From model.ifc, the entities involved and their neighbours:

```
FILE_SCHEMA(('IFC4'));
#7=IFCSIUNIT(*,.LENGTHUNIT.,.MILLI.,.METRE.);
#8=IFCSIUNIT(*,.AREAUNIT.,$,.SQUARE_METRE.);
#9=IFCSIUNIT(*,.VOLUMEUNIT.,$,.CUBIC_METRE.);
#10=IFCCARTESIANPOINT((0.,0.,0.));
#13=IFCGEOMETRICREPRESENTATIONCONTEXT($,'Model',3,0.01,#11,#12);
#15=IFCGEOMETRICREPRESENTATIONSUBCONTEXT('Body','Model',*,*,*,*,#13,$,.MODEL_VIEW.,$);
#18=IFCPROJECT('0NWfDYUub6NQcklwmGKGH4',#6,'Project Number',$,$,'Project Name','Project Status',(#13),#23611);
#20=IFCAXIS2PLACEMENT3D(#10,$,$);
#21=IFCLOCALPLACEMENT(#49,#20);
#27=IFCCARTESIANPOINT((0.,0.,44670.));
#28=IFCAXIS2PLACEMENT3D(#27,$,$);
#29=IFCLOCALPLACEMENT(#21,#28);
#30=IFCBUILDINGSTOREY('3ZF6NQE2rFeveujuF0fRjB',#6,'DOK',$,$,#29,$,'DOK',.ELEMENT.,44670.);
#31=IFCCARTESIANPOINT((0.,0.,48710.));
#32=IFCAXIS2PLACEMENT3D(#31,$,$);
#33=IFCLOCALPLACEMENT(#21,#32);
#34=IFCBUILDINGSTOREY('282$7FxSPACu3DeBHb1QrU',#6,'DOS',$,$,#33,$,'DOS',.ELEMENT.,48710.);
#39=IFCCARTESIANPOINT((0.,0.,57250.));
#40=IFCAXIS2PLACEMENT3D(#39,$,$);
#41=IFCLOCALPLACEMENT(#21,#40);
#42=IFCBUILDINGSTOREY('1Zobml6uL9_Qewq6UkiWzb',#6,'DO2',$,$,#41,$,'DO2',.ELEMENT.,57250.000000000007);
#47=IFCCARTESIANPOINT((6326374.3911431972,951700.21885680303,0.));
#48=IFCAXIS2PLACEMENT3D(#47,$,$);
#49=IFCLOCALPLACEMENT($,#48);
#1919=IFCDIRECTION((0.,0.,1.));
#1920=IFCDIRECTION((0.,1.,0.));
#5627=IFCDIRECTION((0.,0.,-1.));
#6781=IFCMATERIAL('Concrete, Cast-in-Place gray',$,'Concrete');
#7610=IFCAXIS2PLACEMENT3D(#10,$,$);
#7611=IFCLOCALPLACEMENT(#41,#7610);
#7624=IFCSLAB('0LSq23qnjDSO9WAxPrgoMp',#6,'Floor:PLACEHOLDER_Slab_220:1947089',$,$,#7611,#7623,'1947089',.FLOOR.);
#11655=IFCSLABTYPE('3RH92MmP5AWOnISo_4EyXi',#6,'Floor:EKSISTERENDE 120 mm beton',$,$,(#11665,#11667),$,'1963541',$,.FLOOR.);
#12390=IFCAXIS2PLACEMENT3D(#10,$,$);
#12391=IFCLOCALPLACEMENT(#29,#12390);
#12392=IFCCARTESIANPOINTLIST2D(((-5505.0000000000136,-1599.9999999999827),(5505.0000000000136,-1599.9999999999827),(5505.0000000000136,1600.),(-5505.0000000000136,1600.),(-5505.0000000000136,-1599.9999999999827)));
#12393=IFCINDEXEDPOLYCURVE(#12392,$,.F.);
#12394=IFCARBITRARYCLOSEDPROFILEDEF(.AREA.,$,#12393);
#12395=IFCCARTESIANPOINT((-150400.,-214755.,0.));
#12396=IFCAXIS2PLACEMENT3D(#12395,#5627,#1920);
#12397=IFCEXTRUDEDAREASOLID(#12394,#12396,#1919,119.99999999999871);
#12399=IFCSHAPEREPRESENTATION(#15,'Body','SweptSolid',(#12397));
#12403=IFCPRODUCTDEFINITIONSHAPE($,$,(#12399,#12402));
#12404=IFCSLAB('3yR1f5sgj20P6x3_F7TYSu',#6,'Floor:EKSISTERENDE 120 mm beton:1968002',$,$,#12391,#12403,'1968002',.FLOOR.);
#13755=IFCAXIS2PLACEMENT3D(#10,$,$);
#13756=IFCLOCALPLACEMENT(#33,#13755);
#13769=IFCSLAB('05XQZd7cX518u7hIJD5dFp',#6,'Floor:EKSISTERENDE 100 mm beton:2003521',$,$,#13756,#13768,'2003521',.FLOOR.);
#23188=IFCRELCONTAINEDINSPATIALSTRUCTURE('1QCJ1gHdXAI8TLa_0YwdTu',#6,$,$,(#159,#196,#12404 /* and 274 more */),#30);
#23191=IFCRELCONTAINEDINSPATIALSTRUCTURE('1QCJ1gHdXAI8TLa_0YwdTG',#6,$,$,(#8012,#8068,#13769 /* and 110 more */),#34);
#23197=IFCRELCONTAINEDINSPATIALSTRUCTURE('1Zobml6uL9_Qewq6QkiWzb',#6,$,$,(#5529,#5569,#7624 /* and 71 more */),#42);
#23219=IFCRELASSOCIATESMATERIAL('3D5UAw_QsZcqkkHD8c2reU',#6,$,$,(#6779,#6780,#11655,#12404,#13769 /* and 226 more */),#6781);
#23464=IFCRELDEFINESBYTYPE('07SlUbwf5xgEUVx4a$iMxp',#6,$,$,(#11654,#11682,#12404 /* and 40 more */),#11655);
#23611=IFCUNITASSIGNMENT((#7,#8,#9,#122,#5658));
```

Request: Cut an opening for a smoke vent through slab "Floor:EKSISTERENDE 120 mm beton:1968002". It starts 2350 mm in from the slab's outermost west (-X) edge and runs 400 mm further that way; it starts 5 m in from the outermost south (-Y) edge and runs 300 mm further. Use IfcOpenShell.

```python
import numpy as np
import ifcopenshell
import ifcopenshell.api.feature
import ifcopenshell.api.geometry
import ifcopenshell.api.root
import ifcopenshell.geom
import ifcopenshell.util.placement
import ifcopenshell.util.representation
import ifcopenshell.util.shape
import ifcopenshell.util.unit

model = ifcopenshell.open("model.ifc")
unit_scale = ifcopenshell.util.unit.calculate_unit_scale(model)
settings = ifcopenshell.geom.settings()


def volume(element):
    """Net volume in cubic metres, openings subtracted."""
    shape = ifcopenshell.geom.create_shape(settings, element)
    return ifcopenshell.util.shape.get_volume(shape.geometry)


slab = model.by_guid("3yR1f5sgj20P6x3_F7TYSu")
before = volume(slab)

# Extent in the slab's own axes, in metres. The edges named are its -X and -Y sides.
slab_shape = ifcopenshell.geom.create_shape(settings, slab)
vertices = ifcopenshell.util.shape.get_vertices(slab_shape.geometry)
x_min, y_min, bottom = vertices.min(axis=0)
top = vertices[:, 2].max()

opening = ifcopenshell.api.root.create_entity(model, ifc_class="IfcOpeningElement", name="Smoke vent opening", predefined_type="OPENING")
context = ifcopenshell.util.representation.get_context(model, "Model", "Body", "MODEL_VIEW")
width, depth = 0.4, 0.3
outline = [(0.0, 0.0), (width, 0.0), (width, depth), (0.0, depth), (0.0, 0.0)]
# Overshoot both faces by 50 mm so the cut is clean.
shape = ifcopenshell.api.geometry.add_slab_representation(
    model, context=context, depth=top - bottom + 0.1, polyline=outline
)
ifcopenshell.api.geometry.assign_representation(model, product=opening, representation=shape)

matrix = ifcopenshell.util.placement.get_local_placement(slab.ObjectPlacement)
matrix[:, 3] = matrix @ np.append(np.array([x_min + 2.35, y_min + 5, bottom - 0.05]) / unit_scale, 1.0)
ifcopenshell.api.geometry.edit_object_placement(model, product=opening, matrix=matrix, is_si=False)
ifcopenshell.api.feature.add_feature(model, feature=opening, element=slab)

after = volume(slab)

print(f"slab volume {before:.3f} -> {after:.3f} m3")

model.write("model-out.ifc")
```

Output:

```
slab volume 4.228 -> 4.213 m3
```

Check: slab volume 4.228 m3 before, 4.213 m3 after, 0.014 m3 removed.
